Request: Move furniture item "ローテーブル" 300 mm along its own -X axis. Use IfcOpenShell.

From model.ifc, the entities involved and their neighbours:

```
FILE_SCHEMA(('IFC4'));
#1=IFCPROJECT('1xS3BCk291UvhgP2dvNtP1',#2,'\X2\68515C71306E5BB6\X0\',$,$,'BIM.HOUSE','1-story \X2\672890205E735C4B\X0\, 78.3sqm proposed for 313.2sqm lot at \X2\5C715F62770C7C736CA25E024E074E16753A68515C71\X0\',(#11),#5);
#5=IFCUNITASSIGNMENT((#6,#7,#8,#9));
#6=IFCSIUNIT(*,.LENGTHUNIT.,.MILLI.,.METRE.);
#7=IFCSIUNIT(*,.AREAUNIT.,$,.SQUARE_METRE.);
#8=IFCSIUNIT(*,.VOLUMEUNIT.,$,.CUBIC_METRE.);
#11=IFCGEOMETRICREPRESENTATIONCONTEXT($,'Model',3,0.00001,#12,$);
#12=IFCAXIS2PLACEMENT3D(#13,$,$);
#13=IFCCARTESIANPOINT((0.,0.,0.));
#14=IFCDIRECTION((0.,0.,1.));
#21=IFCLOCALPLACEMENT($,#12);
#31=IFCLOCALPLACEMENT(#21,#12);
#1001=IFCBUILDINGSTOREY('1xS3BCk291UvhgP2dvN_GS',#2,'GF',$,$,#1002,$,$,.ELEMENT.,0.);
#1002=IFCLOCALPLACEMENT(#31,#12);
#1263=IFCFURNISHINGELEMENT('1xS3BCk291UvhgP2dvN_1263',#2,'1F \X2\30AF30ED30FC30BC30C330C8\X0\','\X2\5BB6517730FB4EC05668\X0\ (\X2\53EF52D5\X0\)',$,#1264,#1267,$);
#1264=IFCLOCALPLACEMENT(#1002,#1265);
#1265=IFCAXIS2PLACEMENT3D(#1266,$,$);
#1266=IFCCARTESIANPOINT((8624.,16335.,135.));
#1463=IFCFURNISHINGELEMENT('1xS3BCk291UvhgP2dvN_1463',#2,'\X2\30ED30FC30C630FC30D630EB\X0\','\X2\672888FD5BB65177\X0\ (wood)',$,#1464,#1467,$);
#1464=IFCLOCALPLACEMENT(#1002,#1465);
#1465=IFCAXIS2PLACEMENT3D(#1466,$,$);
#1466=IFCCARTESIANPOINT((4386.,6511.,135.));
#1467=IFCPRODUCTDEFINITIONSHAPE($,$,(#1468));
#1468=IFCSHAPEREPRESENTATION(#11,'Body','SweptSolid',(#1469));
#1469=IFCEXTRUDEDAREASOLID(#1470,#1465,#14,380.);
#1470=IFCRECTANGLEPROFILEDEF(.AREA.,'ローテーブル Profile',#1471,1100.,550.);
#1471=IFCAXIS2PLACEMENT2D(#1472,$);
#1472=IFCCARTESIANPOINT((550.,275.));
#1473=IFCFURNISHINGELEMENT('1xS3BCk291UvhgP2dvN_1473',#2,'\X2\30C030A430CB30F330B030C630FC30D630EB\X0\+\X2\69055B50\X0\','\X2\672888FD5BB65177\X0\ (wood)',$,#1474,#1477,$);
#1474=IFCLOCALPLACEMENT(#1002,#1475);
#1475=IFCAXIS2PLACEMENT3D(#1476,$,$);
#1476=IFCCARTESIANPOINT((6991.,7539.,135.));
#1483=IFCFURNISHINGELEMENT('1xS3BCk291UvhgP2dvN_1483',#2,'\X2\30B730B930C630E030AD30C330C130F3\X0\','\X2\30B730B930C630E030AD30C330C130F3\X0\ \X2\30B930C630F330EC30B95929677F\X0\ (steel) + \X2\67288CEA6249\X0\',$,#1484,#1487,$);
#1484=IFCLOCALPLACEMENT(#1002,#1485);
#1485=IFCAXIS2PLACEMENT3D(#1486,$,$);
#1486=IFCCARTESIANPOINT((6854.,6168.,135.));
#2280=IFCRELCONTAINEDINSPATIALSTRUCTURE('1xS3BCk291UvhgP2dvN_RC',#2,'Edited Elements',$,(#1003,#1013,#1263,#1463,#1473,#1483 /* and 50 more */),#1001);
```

```python
import ifcopenshell
import ifcopenshell.api.geometry
import ifcopenshell.util.placement
import ifcopenshell.util.unit

model = ifcopenshell.open("model.ifc")
unit_scale = ifcopenshell.util.unit.calculate_unit_scale(model)

item = model.by_guid("1xS3BCk291UvhgP2dvN_1463")
matrix = ifcopenshell.util.placement.get_local_placement(item.ObjectPlacement)
matrix[:3, 3] -= matrix[:3, 0] * 0.3 / unit_scale
ifcopenshell.api.geometry.edit_object_placement(model, product=item, matrix=matrix, is_si=False)

print(ifcopenshell.util.placement.get_local_placement(item.ObjectPlacement).round(3) + 0.0)

model.write("model_v2.ifc")
```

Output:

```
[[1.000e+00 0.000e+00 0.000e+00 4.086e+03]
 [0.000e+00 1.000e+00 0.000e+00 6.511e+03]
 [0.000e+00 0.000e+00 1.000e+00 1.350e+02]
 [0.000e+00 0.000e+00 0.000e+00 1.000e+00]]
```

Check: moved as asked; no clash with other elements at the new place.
